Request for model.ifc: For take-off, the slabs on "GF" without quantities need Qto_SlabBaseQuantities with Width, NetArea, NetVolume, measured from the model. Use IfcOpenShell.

First a look at what the model holds.

```python
import ifcopenshell
import ifcopenshell.util.element
import ifcopenshell.util.unit

model = ifcopenshell.open("model.ifc")
print(model.schema)
for unit_type in ("LENGTHUNIT", "AREAUNIT", "VOLUMEUNIT"):
    print(unit_type, ifcopenshell.util.unit.calculate_unit_scale(model, unit_type))
storey = next(s for s in model.by_type("IfcBuildingStorey") if s.Name == "GF")
slabs = [e for e in ifcopenshell.util.element.get_decomposition(storey) if e.is_a("IfcSlab")]
for e in sorted(slabs, key=lambda e: e.id()):
    print(e.id(), e.is_a(), e.Name, list(ifcopenshell.util.element.get_psets(e, qtos_only=True)), sep=" | ")
```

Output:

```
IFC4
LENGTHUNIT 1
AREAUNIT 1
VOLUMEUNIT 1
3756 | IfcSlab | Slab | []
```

```python
import ifcopenshell
import ifcopenshell.api.pset
import ifcopenshell.geom
import ifcopenshell.util.element
import ifcopenshell.util.shape
import ifcopenshell.util.unit

model = ifcopenshell.open("model.ifc")
unit_scale = ifcopenshell.util.unit.calculate_unit_scale(model)
area_scale = ifcopenshell.util.unit.calculate_unit_scale(model, "AREAUNIT")
volume_scale = ifcopenshell.util.unit.calculate_unit_scale(model, "VOLUMEUNIT")
settings = ifcopenshell.geom.settings()

storey = next(s for s in model.by_type("IfcBuildingStorey") if s.Name == "GF")
slabs = [e for e in ifcopenshell.util.element.get_decomposition(storey) if e.is_a("IfcSlab")]

for e in sorted(slabs, key=lambda e: e.id()):
    if ifcopenshell.util.element.get_psets(e, qtos_only=True, should_inherit=False):
        continue
    # Geometry comes back in metres, in the element's own axes.
    shape = ifcopenshell.geom.create_shape(settings, e)
    values = {
        "Width": ifcopenshell.util.shape.get_z(shape.geometry) / unit_scale,
        "NetArea": ifcopenshell.util.shape.get_footprint_area(shape.geometry) / area_scale,
        "NetVolume": ifcopenshell.util.shape.get_volume(shape.geometry) / volume_scale,
    }
    qto = ifcopenshell.api.pset.add_qto(model, product=e, name="Qto_SlabBaseQuantities")
    ifcopenshell.api.pset.edit_qto(model, qto=qto, properties=values)
    print(e.id(), {k: round(v, 3) for k, v in values.items()})

model.write("model_rev.ifc")
```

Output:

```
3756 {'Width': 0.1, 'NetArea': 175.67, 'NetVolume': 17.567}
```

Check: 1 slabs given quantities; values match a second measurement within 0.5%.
